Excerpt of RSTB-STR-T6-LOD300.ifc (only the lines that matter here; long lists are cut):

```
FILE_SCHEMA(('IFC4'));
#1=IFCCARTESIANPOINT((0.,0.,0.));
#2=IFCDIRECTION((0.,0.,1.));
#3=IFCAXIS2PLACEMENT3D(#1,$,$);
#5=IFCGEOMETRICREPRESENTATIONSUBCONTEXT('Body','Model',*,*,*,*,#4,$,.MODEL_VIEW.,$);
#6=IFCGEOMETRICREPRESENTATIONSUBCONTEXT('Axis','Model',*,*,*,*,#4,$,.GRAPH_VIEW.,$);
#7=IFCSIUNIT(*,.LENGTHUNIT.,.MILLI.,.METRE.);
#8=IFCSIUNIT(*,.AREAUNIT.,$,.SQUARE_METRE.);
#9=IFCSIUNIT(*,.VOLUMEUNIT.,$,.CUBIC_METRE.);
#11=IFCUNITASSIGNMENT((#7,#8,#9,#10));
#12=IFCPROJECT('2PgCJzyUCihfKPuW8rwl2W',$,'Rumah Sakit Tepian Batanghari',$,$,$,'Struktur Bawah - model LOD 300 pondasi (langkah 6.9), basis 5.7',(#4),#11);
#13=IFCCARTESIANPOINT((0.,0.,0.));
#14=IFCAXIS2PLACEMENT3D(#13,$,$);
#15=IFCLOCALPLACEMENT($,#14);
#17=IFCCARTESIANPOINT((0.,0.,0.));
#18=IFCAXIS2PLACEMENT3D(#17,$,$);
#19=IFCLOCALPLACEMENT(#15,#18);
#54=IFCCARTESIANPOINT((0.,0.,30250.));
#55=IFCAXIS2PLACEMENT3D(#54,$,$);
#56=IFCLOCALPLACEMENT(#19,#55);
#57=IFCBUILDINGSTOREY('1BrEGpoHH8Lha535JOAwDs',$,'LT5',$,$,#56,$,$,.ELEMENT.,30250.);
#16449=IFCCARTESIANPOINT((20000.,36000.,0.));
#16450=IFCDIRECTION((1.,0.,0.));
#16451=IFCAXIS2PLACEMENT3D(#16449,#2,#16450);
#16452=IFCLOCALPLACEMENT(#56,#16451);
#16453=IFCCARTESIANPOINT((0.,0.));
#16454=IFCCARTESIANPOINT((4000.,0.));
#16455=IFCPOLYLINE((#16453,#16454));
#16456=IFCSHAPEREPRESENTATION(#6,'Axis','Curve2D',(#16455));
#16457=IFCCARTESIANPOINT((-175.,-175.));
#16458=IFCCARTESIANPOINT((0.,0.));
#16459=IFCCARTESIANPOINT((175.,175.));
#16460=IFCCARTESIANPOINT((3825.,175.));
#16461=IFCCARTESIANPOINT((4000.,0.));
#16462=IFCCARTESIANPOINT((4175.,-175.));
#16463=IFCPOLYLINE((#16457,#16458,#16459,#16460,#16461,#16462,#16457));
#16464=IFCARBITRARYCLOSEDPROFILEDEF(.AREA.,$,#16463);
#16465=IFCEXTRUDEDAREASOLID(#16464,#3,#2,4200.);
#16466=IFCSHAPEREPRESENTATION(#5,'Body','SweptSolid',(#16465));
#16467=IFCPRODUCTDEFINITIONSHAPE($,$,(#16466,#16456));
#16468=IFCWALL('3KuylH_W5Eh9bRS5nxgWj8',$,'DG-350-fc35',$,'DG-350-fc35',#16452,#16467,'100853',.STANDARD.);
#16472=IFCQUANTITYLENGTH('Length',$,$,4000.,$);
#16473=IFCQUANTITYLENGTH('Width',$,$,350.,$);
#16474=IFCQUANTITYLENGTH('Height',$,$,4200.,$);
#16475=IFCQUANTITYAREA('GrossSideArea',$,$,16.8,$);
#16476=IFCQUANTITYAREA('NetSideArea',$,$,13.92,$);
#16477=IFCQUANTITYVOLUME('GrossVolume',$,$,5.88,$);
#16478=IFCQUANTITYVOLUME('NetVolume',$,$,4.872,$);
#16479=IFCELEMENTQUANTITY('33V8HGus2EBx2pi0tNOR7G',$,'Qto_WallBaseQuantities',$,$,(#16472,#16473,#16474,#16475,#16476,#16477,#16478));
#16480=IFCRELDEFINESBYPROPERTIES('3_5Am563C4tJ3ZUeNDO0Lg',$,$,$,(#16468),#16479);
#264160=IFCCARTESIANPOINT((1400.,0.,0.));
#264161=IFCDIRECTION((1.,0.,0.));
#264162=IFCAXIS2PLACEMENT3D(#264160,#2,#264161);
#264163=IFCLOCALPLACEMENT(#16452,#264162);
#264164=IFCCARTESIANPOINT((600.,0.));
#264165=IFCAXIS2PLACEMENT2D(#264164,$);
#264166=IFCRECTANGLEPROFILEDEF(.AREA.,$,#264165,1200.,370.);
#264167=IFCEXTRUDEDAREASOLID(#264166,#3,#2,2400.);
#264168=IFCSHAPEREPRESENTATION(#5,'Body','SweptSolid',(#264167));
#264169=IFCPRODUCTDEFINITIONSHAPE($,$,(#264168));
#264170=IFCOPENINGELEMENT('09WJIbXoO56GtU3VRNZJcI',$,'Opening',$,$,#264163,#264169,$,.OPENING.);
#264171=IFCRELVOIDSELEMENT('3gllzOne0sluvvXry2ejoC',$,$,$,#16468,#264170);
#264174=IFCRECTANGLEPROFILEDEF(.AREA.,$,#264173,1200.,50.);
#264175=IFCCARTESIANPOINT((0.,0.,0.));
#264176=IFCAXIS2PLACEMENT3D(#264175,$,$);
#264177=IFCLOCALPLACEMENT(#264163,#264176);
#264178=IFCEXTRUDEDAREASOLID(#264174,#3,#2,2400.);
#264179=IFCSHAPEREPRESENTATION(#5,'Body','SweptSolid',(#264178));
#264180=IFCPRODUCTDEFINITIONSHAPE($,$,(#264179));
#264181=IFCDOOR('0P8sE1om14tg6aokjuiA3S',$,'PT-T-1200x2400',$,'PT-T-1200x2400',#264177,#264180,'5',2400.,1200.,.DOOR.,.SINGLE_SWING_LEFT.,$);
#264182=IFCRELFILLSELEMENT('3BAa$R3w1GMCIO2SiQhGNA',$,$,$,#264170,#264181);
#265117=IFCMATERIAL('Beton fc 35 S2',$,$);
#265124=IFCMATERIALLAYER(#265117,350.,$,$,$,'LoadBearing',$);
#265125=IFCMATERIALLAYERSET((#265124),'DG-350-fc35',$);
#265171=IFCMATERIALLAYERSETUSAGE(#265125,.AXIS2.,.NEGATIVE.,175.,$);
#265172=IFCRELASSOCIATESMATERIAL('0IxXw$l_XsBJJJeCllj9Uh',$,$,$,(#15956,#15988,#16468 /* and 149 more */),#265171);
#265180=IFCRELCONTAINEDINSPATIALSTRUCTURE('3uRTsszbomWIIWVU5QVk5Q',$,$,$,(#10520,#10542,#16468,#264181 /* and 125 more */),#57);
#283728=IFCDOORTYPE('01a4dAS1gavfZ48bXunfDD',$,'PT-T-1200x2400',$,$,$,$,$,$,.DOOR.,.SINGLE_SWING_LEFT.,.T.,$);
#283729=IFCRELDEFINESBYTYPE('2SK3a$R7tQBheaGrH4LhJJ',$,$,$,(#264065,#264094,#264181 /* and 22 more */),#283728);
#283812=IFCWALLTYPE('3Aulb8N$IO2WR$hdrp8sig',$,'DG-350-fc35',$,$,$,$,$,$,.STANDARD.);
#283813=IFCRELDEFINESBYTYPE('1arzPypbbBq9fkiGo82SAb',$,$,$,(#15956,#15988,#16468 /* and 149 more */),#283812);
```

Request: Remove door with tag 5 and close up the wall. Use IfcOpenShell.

```python
import ifcopenshell
import ifcopenshell.api.feature
import ifcopenshell.api.pset
import ifcopenshell.api.root
import ifcopenshell.geom
import ifcopenshell.util.element
import ifcopenshell.util.shape
import ifcopenshell.util.unit

model = ifcopenshell.open("RSTB-STR-T6-LOD300.ifc")
area_scale = ifcopenshell.util.unit.calculate_unit_scale(model, "AREAUNIT")
volume_scale = ifcopenshell.util.unit.calculate_unit_scale(model, "VOLUMEUNIT")
settings = ifcopenshell.geom.settings()


def volume(element):
    """Net volume in cubic metres, openings subtracted."""
    shape = ifcopenshell.geom.create_shape(settings, element)
    return ifcopenshell.util.shape.get_volume(shape.geometry)


door = model.by_guid("0P8sE1om14tg6aokjuiA3S")
opening = door.FillsVoids[0].RelatingOpeningElement
wall = opening.VoidsElements[0].RelatingBuildingElement
before = volume(wall)

ifcopenshell.api.root.remove_product(model, product=door)
ifcopenshell.api.feature.remove_feature(model, feature=opening)

after = volume(wall)
thickness = 0.35  # wall thickness in metres

# Update the wall's stored quantities.
qto = model.by_id(ifcopenshell.util.element.get_pset(wall, "Qto_WallBaseQuantities", should_inherit=False)["id"])
ifcopenshell.api.pset.edit_qto(model, qto=qto, properties={
    "NetSideArea": after / thickness / area_scale,
    "NetVolume": after / volume_scale,
})

print(f"wall volume {before:.3f} -> {after:.3f} m3")

model.write("RSTB-STR-T6-LOD300_v2.ifc")
```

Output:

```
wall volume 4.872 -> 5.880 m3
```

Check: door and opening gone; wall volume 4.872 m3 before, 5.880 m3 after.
